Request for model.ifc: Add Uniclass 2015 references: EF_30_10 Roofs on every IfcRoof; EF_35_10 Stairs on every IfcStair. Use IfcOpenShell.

First a look at what the model holds.

```python
import ifcopenshell

model = ifcopenshell.open("model.ifc")
print(model.schema)
print("classifications:", [c.Name for c in model.by_type("IfcClassification")])
for ifc_class in ("IfcDoor", "IfcRoof", "IfcStair", "IfcWall", "IfcWindow"):
    print(ifc_class, len(model.by_type(ifc_class)))
```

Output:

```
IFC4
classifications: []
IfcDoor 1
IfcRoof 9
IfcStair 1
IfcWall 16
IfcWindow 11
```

```python
import ifcopenshell
import ifcopenshell.api.classification

model = ifcopenshell.open("model.ifc")

system = ifcopenshell.api.classification.add_classification(model, classification="Uniclass 2015")

codes = {
    "IfcRoof": ("EF_30_10", "Roofs"),
    "IfcStair": ("EF_35_10", "Stairs"),
}
for ifc_class, (code, name) in codes.items():
    products = model.by_type(ifc_class)
    ifcopenshell.api.classification.add_reference(
        model, products=products, classification=system, identification=code, name=name
    )
    print(code, len(products))

model.write("model_edited.ifc")
```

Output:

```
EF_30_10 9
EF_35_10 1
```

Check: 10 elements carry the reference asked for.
